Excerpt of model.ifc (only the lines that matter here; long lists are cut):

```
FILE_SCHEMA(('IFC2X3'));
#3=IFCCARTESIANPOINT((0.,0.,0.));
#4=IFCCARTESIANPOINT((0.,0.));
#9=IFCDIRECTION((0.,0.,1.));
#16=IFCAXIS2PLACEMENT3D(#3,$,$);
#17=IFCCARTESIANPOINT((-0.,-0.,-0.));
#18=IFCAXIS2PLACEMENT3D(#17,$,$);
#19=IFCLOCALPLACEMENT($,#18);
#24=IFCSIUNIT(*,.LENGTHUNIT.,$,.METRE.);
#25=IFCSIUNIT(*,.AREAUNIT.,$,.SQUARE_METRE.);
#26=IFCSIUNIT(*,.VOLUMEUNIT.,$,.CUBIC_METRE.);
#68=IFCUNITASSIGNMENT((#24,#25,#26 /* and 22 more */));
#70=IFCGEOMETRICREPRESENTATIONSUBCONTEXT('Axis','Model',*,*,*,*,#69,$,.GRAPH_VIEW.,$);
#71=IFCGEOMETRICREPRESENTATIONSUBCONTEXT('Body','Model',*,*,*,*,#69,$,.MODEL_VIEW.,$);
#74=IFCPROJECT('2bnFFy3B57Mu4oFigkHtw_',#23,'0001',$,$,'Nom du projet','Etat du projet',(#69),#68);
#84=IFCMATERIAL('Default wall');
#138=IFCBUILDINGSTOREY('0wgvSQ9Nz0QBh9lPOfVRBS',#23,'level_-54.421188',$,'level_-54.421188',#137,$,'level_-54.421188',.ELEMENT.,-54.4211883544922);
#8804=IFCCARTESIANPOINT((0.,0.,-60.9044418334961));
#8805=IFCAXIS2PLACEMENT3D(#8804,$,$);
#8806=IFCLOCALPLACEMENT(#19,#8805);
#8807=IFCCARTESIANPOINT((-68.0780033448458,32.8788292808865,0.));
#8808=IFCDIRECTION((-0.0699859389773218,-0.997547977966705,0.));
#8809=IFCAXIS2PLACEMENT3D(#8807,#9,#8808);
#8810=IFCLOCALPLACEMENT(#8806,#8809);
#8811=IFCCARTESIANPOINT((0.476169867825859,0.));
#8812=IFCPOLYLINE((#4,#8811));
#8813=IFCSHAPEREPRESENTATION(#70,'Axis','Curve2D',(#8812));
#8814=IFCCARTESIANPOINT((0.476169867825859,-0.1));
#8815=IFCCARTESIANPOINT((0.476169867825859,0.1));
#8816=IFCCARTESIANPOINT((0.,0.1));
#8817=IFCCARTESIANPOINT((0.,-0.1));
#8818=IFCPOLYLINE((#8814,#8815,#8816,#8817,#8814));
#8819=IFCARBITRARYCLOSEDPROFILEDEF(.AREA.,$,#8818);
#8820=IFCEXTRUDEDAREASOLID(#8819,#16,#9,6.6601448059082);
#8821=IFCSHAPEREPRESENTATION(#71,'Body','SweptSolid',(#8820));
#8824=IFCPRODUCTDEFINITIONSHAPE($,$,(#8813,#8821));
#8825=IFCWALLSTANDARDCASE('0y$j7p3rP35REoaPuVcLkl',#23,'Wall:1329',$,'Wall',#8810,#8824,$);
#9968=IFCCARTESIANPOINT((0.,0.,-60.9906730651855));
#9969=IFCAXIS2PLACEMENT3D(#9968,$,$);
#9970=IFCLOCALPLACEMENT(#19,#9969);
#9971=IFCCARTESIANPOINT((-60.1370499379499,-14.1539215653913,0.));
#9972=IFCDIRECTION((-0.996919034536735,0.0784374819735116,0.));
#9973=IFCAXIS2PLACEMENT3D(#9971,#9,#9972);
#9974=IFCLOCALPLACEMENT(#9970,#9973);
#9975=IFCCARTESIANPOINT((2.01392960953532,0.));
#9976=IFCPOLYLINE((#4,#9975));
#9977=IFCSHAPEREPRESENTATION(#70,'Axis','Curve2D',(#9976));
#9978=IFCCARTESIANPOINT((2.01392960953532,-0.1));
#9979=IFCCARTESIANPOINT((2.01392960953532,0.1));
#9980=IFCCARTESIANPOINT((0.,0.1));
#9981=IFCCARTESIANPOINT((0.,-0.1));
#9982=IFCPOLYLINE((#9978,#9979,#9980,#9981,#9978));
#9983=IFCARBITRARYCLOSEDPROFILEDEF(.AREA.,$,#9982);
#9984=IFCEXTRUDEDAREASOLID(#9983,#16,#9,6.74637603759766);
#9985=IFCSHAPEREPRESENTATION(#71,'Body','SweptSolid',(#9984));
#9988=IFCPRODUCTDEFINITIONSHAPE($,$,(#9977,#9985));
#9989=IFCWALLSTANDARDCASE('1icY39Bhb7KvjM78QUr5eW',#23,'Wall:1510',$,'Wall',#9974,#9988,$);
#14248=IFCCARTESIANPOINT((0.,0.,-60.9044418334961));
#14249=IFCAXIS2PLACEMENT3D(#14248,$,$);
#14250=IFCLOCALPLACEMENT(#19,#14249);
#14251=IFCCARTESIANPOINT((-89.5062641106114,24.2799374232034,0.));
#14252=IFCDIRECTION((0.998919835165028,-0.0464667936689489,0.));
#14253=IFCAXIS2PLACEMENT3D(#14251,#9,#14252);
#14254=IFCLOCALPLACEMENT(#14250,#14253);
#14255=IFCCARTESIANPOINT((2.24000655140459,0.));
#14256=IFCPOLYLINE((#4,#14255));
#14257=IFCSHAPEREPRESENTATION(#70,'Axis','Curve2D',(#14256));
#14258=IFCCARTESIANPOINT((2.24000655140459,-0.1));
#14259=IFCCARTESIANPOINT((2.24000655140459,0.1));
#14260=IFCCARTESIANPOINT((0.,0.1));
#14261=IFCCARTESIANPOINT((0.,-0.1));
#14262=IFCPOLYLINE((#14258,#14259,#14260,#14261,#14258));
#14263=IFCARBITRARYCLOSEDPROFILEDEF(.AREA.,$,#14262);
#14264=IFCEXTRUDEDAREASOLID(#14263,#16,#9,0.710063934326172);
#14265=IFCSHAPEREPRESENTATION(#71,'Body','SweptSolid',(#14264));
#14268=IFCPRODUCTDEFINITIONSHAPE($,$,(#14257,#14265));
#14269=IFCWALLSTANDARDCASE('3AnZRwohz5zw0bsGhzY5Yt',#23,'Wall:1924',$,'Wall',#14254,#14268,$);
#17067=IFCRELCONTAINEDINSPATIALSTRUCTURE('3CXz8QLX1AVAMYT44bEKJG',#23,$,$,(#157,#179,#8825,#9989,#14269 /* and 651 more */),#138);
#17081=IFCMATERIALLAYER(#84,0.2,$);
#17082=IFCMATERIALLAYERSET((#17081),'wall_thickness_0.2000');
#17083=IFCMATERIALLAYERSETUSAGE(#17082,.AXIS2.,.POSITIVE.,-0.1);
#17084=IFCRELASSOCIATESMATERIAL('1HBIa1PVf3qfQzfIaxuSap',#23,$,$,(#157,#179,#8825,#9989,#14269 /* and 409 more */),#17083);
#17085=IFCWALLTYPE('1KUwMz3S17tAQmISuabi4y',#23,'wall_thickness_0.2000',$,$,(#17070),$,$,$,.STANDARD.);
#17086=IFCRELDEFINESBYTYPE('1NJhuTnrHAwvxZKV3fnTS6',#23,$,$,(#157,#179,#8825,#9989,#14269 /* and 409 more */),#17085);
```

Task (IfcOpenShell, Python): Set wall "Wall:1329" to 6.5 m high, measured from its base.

```python
import ifcopenshell
import ifcopenshell.geom
import ifcopenshell.util.representation
import ifcopenshell.util.shape
import ifcopenshell.util.unit

model = ifcopenshell.open("model.ifc")
unit_scale = ifcopenshell.util.unit.calculate_unit_scale(model)
settings = ifcopenshell.geom.settings()


def volume(element):
    """Net volume in cubic metres, openings subtracted."""
    shape = ifcopenshell.geom.create_shape(settings, element)
    return ifcopenshell.util.shape.get_volume(shape.geometry)


wall = model.by_id(8825)
before = volume(wall)

body = ifcopenshell.util.representation.get_representation(wall, "Model", "Body")
solid = body.Items[0]
old_height = solid.Depth
solid.Depth = 6.5 / unit_scale
after = volume(wall)

print(f"height {old_height:g} -> {solid.Depth:g}, volume {before:.3f} -> {after:.3f} m3")

model.write("model_rev.ifc")
```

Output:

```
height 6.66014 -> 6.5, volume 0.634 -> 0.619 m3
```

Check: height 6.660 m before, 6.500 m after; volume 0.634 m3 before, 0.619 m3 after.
